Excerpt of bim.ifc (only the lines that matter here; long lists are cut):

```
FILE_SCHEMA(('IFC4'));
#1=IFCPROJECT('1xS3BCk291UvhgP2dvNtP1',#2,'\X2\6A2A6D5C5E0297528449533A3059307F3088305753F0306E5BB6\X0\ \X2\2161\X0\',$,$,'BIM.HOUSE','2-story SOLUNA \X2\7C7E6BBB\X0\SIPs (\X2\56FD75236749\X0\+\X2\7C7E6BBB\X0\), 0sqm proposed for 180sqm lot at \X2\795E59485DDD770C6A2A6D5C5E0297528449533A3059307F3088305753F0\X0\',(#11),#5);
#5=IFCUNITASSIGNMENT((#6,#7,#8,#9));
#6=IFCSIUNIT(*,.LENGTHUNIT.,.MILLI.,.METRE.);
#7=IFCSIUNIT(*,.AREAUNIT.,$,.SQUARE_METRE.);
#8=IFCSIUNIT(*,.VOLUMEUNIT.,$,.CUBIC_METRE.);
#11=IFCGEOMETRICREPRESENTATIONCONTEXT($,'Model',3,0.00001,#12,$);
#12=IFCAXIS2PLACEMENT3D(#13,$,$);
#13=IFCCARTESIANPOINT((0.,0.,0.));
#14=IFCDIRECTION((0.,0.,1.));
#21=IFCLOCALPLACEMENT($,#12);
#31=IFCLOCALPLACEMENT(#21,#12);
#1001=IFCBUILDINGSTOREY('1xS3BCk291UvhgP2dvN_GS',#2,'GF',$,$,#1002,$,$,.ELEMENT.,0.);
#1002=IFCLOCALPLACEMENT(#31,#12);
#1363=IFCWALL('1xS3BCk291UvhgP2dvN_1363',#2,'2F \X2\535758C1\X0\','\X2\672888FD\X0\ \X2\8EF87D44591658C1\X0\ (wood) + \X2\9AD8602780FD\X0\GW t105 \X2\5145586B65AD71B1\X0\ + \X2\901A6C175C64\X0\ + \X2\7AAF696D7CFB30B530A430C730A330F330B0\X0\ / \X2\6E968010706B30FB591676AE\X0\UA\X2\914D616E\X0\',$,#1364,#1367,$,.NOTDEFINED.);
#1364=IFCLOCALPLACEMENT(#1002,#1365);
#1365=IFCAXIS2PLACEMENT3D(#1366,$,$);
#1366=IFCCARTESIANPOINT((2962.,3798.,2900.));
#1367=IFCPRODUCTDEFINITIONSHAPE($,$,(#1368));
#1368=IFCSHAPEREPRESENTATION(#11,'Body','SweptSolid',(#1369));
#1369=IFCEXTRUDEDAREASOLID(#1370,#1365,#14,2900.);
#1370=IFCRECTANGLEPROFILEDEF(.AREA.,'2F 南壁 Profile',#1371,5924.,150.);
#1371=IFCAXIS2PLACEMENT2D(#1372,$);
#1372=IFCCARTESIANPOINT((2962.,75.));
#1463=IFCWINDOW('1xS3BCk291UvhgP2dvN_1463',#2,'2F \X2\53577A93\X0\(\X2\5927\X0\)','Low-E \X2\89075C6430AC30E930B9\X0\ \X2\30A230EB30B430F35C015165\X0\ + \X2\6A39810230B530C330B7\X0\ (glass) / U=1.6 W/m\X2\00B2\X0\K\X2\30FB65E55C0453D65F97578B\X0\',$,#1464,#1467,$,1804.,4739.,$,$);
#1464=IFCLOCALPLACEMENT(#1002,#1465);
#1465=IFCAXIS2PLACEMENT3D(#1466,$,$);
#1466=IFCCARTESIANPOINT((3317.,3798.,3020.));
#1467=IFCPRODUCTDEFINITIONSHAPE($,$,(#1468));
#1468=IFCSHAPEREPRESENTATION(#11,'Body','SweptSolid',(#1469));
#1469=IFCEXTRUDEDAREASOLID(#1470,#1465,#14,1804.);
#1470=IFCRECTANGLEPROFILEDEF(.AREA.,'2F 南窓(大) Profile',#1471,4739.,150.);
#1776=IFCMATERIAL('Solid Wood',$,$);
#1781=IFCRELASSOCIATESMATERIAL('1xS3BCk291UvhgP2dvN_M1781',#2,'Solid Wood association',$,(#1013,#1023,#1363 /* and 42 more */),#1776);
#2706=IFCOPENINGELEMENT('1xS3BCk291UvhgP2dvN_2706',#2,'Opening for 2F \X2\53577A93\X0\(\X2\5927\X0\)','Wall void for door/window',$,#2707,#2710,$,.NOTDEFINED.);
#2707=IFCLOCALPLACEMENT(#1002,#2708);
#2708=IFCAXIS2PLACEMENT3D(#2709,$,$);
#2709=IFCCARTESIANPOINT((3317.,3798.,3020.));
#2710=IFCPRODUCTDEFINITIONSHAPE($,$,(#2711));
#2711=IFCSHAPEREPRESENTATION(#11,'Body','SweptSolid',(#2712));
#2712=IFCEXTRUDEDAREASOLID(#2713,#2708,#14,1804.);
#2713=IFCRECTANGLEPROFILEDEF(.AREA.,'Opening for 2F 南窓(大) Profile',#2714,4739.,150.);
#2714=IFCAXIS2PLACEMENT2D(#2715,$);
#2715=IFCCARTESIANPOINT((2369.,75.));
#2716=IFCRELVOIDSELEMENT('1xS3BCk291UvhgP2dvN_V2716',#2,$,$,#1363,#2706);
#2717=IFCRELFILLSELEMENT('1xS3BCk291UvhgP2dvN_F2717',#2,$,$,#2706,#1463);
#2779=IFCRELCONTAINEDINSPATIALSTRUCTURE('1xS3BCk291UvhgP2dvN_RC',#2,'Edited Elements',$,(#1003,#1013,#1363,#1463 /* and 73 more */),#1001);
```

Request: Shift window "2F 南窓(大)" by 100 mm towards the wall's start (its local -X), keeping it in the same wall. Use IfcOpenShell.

```python
import ifcopenshell
import ifcopenshell.api.geometry
import ifcopenshell.util.placement

model = ifcopenshell.open("bim.ifc")

window = model.by_id(1463)
opening = window.FillsVoids[0].RelatingOpeningElement
wall = opening.VoidsElements[0].RelatingBuildingElement

wall_matrix = ifcopenshell.util.placement.get_local_placement(wall.ObjectPlacement)
shift = wall_matrix[:3, 0] * -100.0
before = ifcopenshell.util.placement.get_local_placement(window.ObjectPlacement)[:3, 3].copy()

# The window is not placed relative to its opening, so move both.
for product in (opening, window):
    matrix = ifcopenshell.util.placement.get_local_placement(product.ObjectPlacement)
    matrix[:3, 3] += shift
    ifcopenshell.api.geometry.edit_object_placement(model, product=product, matrix=matrix, is_si=False)

after = ifcopenshell.util.placement.get_local_placement(window.ObjectPlacement)[:3, 3]
print("window moved by", (after - before).round(3) + 0.0)

model.write("bim_edited.ifc")
```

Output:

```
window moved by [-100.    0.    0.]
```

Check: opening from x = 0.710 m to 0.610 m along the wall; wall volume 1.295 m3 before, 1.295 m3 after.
